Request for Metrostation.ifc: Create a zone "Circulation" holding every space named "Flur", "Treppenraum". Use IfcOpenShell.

First a look at what the model holds.

```python
import ifcopenshell

model = ifcopenshell.open("Metrostation.ifc")
print(model.schema)
seen = {}
for space in model.by_type("IfcSpace"):
    seen[space.LongName] = seen.get(space.LongName, 0) + 1
for name, count in sorted(seen.items(), key=str):
    print(count, "x", name)
print("zones:", [z.Name for z in model.by_type("IfcZone")][:20])
```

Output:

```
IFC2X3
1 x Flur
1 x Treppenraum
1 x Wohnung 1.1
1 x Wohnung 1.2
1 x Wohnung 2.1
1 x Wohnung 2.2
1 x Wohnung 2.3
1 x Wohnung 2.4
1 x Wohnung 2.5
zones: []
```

```python
import ifcopenshell
import ifcopenshell.api.group
import ifcopenshell.api.root

model = ifcopenshell.open("Metrostation.ifc")

names = {"Flur", "Treppenraum"}
spaces = [s for s in model.by_type("IfcSpace") if s.LongName in names]

zone = ifcopenshell.api.root.create_entity(model, ifc_class="IfcZone", name="Circulation")
ifcopenshell.api.group.assign_group(model, products=spaces, group=zone)
print(len(spaces), "spaces in", zone.Name)

model.write("Metrostation_edited.ifc")
```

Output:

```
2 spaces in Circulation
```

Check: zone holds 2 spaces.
